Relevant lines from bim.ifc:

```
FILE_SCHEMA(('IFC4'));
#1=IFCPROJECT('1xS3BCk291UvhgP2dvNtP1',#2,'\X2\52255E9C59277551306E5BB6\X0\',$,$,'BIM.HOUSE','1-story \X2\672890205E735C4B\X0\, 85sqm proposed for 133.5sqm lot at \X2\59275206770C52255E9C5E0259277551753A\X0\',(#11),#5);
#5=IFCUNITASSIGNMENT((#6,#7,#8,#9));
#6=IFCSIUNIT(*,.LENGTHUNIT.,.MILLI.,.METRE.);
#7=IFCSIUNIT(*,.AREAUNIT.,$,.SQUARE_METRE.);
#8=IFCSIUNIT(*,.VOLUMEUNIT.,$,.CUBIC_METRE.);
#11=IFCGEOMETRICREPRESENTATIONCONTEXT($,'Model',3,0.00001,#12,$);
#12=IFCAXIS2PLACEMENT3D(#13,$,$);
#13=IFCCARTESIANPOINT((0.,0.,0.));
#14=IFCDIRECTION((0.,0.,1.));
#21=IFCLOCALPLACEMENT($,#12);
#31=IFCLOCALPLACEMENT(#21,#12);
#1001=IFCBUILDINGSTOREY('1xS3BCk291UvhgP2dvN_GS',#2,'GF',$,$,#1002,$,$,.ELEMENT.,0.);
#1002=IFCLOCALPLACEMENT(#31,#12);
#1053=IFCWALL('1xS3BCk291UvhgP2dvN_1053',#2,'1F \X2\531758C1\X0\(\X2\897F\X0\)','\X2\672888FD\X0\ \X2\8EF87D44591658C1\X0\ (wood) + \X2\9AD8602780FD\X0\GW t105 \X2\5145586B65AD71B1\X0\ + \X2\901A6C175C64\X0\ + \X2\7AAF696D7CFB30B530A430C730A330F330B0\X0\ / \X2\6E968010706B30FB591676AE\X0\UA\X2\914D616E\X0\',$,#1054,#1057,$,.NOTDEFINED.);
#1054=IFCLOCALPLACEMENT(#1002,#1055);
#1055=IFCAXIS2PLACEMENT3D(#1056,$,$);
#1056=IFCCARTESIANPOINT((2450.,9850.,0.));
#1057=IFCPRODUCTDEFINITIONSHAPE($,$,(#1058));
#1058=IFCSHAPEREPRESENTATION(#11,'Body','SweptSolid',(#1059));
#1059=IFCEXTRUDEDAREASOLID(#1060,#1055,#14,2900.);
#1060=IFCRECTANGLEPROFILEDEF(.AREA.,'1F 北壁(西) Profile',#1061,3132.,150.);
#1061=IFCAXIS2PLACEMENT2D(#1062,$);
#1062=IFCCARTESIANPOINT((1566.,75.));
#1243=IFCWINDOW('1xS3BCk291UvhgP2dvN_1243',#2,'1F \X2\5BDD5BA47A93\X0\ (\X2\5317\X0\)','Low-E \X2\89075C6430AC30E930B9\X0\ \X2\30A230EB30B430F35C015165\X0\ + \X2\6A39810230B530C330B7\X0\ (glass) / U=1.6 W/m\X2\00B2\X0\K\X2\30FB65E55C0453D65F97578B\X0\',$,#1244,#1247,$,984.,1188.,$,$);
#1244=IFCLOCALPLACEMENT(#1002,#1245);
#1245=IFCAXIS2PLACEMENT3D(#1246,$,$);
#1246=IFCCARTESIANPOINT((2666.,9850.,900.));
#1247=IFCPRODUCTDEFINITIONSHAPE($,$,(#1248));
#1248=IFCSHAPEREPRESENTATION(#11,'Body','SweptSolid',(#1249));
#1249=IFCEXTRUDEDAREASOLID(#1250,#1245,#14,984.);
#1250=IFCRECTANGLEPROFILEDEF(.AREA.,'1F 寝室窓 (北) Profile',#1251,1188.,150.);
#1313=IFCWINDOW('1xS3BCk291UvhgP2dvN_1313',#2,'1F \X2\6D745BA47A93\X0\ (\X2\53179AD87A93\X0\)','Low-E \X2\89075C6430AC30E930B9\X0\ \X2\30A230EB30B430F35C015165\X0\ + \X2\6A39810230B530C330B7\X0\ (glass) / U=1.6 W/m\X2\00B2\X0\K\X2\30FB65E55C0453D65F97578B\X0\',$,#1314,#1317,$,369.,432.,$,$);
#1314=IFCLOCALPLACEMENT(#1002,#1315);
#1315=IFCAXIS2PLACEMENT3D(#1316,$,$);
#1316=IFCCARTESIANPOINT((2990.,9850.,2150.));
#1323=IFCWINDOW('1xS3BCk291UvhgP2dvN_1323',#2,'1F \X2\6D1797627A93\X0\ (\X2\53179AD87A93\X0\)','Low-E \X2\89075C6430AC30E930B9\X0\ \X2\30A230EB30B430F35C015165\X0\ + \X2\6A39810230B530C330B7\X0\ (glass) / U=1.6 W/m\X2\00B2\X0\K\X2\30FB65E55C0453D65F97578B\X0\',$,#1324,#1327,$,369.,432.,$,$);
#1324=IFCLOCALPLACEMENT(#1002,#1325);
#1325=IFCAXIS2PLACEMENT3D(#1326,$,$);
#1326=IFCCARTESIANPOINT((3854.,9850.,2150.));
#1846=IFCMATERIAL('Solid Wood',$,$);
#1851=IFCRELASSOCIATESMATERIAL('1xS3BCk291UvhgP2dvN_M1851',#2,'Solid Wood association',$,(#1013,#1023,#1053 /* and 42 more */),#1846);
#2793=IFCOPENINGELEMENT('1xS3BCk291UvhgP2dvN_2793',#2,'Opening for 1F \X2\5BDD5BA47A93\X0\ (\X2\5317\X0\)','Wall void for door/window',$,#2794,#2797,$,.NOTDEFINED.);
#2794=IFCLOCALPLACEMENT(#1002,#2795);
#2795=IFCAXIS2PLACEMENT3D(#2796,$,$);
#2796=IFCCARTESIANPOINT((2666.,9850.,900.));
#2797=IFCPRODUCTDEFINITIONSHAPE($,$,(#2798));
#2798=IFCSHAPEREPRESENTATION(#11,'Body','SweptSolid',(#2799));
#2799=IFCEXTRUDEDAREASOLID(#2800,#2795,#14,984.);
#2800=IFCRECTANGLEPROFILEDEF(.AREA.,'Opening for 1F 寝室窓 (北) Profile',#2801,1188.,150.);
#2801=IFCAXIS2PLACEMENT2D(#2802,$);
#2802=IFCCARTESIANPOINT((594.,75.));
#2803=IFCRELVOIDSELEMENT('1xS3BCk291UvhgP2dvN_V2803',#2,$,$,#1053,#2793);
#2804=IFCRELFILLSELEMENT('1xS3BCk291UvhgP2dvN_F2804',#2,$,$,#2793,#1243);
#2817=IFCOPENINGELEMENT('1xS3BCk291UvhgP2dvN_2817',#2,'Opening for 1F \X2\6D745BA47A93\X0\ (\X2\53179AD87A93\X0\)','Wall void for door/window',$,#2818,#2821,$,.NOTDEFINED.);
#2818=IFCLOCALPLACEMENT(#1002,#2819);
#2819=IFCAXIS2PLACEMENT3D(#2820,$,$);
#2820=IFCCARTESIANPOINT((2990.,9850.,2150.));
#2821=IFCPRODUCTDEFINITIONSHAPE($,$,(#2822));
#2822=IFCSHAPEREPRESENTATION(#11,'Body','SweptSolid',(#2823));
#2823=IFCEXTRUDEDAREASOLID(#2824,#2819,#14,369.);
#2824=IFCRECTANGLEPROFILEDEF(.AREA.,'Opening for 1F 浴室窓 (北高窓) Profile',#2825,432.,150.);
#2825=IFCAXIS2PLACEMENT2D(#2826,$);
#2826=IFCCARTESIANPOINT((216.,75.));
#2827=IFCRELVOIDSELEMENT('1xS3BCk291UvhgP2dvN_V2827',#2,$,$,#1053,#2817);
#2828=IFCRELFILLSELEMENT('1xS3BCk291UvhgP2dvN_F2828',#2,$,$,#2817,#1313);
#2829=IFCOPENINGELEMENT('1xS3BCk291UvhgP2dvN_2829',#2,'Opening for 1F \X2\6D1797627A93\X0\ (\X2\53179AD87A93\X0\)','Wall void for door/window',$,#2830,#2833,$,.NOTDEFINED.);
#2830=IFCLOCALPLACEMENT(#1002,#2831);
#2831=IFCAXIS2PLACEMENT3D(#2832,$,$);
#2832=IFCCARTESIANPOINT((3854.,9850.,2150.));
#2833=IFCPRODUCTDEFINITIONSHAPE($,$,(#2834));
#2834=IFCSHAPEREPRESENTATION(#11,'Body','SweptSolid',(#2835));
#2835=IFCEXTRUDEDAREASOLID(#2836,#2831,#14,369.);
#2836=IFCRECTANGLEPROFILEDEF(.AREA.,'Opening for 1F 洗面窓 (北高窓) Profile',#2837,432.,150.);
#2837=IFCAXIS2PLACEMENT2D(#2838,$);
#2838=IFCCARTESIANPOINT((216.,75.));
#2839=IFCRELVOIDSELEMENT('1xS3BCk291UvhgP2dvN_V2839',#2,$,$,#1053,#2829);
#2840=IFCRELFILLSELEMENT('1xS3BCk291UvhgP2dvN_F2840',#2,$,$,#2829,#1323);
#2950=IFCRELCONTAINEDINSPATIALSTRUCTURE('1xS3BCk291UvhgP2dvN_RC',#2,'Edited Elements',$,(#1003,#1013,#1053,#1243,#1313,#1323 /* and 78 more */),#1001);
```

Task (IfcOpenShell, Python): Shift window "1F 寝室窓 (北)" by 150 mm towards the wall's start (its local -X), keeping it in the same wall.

```python
import ifcopenshell
import ifcopenshell.api.geometry
import ifcopenshell.util.placement
import ifcopenshell.util.unit

model = ifcopenshell.open("bim.ifc")
unit_scale = ifcopenshell.util.unit.calculate_unit_scale(model)

window = model.by_guid("1xS3BCk291UvhgP2dvN_1243")
opening = window.FillsVoids[0].RelatingOpeningElement
wall = opening.VoidsElements[0].RelatingBuildingElement

wall_matrix = ifcopenshell.util.placement.get_local_placement(wall.ObjectPlacement)
shift = wall_matrix[:3, 0] * -0.15 / unit_scale
before = ifcopenshell.util.placement.get_local_placement(window.ObjectPlacement)[:3, 3].copy()

# The window is not placed relative to its opening, so move both.
for product in (opening, window):
    matrix = ifcopenshell.util.placement.get_local_placement(product.ObjectPlacement)
    matrix[:3, 3] += shift
    ifcopenshell.api.geometry.edit_object_placement(model, product=product, matrix=matrix, is_si=False)

after = ifcopenshell.util.placement.get_local_placement(window.ObjectPlacement)[:3, 3]
print("window moved by", (after - before).round(3) + 0.0)

model.write("bim_updated.ifc")
```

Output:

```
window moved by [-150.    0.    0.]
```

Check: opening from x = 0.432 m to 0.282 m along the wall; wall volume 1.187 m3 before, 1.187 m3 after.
